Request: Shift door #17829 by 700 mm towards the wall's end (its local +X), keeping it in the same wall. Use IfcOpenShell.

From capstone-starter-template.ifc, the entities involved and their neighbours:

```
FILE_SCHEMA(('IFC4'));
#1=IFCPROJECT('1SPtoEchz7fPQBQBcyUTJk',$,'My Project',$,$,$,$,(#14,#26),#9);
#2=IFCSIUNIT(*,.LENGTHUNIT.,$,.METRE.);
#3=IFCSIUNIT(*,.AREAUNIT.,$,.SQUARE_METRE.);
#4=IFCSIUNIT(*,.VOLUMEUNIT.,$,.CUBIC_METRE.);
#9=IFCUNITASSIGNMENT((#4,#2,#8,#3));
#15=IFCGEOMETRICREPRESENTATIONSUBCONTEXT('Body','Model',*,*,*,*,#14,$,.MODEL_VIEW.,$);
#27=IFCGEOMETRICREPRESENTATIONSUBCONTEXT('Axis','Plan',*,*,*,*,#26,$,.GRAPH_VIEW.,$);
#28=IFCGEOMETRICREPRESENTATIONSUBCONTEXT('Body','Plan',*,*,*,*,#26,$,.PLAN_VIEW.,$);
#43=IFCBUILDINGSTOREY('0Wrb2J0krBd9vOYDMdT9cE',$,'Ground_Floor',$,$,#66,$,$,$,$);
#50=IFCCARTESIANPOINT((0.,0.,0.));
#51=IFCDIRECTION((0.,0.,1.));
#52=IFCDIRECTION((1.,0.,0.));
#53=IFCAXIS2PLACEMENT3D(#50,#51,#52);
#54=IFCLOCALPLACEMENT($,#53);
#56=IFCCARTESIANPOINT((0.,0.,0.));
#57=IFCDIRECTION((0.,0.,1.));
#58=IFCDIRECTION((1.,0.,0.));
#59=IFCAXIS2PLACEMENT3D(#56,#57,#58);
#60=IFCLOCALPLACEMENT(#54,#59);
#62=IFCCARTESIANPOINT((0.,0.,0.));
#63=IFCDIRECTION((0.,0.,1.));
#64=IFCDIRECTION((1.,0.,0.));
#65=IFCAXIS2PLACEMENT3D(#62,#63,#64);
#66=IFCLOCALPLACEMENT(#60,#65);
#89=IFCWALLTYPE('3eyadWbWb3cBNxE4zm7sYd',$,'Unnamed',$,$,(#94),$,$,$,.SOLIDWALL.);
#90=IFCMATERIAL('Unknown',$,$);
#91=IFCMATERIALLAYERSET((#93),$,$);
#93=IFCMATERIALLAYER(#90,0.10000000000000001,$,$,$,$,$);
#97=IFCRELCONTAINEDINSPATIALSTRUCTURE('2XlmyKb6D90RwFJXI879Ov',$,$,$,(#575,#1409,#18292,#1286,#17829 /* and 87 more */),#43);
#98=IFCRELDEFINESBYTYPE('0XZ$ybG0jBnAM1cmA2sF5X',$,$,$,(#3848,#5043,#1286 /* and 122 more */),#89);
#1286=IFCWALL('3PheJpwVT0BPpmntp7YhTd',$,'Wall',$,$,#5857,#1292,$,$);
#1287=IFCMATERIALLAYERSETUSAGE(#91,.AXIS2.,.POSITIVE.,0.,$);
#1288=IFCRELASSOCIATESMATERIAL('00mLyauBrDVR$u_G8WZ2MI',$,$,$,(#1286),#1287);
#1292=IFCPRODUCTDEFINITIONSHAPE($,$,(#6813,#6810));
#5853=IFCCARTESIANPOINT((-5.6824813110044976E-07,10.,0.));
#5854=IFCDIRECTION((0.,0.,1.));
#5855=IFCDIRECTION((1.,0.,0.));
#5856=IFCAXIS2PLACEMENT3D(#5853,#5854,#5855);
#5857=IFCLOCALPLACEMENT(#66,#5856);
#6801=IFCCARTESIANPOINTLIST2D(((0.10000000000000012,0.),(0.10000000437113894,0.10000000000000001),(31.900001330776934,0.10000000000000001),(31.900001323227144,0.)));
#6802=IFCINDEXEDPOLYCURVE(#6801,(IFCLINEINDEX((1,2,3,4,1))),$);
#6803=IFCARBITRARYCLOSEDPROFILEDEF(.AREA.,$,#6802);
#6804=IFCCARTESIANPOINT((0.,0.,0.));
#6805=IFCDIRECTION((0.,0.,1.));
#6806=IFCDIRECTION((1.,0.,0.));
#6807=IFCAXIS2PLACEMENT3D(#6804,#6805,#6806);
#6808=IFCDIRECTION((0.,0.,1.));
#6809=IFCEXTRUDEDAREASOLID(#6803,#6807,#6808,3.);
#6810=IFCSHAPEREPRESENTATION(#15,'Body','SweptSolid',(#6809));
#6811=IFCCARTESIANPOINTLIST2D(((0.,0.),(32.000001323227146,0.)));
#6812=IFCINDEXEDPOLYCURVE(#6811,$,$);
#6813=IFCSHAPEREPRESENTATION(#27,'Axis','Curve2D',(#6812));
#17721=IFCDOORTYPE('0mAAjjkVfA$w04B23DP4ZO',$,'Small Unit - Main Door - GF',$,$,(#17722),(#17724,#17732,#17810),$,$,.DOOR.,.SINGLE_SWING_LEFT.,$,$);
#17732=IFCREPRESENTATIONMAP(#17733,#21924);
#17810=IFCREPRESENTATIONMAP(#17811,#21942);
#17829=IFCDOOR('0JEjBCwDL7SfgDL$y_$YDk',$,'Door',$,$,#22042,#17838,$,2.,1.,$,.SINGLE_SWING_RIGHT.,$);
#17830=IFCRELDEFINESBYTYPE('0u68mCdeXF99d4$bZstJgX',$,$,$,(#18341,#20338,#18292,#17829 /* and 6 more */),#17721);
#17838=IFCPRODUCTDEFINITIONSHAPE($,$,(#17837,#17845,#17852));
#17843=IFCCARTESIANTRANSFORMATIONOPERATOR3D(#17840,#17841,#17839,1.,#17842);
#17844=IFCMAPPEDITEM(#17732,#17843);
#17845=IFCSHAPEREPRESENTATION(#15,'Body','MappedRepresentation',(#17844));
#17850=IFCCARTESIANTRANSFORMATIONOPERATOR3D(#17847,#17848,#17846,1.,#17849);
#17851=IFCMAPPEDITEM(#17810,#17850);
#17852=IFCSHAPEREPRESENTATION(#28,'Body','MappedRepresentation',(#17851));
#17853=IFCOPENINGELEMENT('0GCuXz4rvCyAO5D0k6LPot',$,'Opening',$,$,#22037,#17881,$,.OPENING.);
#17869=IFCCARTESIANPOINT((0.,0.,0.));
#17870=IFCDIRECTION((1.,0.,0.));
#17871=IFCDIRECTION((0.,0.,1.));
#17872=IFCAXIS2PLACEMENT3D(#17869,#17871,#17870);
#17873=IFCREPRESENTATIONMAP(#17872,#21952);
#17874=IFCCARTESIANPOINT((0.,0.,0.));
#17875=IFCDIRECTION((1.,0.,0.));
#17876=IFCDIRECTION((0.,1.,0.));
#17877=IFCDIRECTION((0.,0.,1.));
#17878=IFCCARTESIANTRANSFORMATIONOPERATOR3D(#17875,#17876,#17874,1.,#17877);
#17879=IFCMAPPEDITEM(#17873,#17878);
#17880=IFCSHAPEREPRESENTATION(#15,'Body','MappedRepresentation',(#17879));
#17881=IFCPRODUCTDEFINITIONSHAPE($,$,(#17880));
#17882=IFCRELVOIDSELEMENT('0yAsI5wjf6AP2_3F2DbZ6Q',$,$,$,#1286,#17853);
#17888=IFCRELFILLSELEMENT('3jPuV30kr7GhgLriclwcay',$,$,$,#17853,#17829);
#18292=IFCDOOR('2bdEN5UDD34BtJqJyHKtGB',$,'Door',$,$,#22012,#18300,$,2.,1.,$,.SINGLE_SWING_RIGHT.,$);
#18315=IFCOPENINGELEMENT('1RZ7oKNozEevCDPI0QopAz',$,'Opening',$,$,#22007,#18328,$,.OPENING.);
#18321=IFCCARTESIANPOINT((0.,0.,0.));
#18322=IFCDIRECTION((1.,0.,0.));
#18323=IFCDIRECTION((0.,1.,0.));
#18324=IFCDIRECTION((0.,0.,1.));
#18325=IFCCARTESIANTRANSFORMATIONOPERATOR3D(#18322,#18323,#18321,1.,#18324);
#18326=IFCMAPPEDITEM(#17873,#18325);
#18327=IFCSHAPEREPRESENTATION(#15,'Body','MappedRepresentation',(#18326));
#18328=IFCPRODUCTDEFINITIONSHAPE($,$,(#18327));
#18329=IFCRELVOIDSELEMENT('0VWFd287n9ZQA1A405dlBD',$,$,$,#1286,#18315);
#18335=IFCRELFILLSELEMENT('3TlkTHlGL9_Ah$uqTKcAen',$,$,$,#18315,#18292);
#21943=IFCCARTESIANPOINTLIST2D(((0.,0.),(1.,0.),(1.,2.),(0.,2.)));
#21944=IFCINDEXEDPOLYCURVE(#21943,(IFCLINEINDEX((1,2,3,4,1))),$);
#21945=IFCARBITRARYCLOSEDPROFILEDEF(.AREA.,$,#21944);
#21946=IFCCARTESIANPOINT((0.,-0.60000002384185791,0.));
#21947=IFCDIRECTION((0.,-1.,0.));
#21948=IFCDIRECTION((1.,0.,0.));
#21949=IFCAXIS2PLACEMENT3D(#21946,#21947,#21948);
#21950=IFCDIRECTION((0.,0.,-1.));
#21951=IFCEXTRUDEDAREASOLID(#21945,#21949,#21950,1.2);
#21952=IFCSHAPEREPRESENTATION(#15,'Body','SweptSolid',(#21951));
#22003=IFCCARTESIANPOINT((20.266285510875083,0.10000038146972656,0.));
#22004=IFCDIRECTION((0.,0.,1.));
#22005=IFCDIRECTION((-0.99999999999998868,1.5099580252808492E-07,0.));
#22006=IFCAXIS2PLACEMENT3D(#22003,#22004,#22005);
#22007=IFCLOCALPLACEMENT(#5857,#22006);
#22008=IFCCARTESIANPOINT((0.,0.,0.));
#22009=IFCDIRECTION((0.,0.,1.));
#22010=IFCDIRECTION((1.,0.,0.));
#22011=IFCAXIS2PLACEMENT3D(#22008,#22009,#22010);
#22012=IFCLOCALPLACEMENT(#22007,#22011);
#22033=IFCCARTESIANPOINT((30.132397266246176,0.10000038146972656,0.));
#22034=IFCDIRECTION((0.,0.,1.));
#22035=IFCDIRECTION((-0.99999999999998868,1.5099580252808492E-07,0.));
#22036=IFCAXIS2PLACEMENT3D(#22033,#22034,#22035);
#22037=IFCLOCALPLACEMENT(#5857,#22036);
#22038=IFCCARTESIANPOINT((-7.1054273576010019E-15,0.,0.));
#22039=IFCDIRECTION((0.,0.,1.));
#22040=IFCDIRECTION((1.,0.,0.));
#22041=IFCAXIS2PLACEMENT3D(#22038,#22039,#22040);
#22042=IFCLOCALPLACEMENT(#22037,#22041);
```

```python
import ifcopenshell
import ifcopenshell.api.geometry
import ifcopenshell.util.placement
import ifcopenshell.util.unit

model = ifcopenshell.open("capstone-starter-template.ifc")
unit_scale = ifcopenshell.util.unit.calculate_unit_scale(model)

door = model.by_guid("0JEjBCwDL7SfgDL$y_$YDk")
opening = door.FillsVoids[0].RelatingOpeningElement
wall = opening.VoidsElements[0].RelatingBuildingElement

wall_matrix = ifcopenshell.util.placement.get_local_placement(wall.ObjectPlacement)
shift = wall_matrix[:3, 0] * 0.7 / unit_scale
before = ifcopenshell.util.placement.get_local_placement(door.ObjectPlacement)[:3, 3].copy()

# The door is placed relative to its opening, so it follows when the opening moves.
matrix = ifcopenshell.util.placement.get_local_placement(opening.ObjectPlacement)
matrix[:3, 3] += shift
ifcopenshell.api.geometry.edit_object_placement(
    model, product=opening, matrix=matrix, is_si=False, should_transform_children=True
)

after = ifcopenshell.util.placement.get_local_placement(door.ObjectPlacement)[:3, 3]
print("door moved by", (after - before).round(3) + 0.0)

model.write("capstone-starter-template_v2.ifc")
```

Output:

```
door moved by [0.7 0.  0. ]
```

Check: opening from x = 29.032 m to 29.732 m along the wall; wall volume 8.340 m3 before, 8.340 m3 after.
